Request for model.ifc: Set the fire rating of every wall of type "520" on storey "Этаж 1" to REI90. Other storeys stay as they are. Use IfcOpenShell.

First a look at what the model holds.

```python
import ifcopenshell
import ifcopenshell.util.element

model = ifcopenshell.open("model.ifc")
print(model.schema)
storey = next(s for s in model.by_type("IfcBuildingStorey") if s.Name == "Этаж 1")
walls = [e for e in ifcopenshell.util.element.get_decomposition(storey) if e.is_a("IfcWall")]
seen = {}
for e in walls:
    element_type = ifcopenshell.util.element.get_type(e)
    key = (element_type.Name if element_type != e and element_type else None, ifcopenshell.util.element.get_pset(e, "Pset_WallCommon", "FireRating"))
    seen[key] = seen.get(key, 0) + 1
for (name, value), count in sorted(seen.items(), key=str):
    print(count, "x", name, "|", value)
```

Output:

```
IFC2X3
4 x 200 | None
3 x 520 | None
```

```python
import ifcopenshell
import ifcopenshell.api.pset
import ifcopenshell.util.element

model = ifcopenshell.open("model.ifc")

storey = next(s for s in model.by_type("IfcBuildingStorey") if s.Name == "Этаж 1")
walls = [e for e in ifcopenshell.util.element.get_decomposition(storey) if e.is_a("IfcWall")]

count = 0
for e in walls:
    element_type = ifcopenshell.util.element.get_type(e)
    if element_type in (None, e) or element_type.Name != "520":
        continue
    # add_pset returns the element's existing set when there is one.
    pset = ifcopenshell.api.pset.add_pset(model, product=e, name="Pset_WallCommon")
    ifcopenshell.api.pset.edit_pset(model, pset=pset, properties={"FireRating": "REI90"})
    count += 1

print(count, "walls updated")

model.write("model-out.ifc")
```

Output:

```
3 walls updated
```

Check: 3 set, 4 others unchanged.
